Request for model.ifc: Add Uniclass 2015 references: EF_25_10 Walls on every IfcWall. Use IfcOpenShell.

First a look at what the model holds.

```python
import ifcopenshell

model = ifcopenshell.open("model.ifc")
print(model.schema)
print("classifications:", [c.Name for c in model.by_type("IfcClassification")])
for ifc_class in ("IfcDoor", "IfcRoof", "IfcStair", "IfcWall", "IfcWindow"):
    print(ifc_class, len(model.by_type(ifc_class)))
```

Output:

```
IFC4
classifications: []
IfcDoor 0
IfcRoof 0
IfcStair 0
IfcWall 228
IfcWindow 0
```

```python
import ifcopenshell
import ifcopenshell.api.classification

model = ifcopenshell.open("model.ifc")

system = ifcopenshell.api.classification.add_classification(model, classification="Uniclass 2015")

codes = {
    "IfcWall": ("EF_25_10", "Walls"),
}
for ifc_class, (code, name) in codes.items():
    products = model.by_type(ifc_class)
    ifcopenshell.api.classification.add_reference(
        model, products=products, classification=system, identification=code, name=name
    )
    print(code, len(products))

model.write("model-out.ifc")
```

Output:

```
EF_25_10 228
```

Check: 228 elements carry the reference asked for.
